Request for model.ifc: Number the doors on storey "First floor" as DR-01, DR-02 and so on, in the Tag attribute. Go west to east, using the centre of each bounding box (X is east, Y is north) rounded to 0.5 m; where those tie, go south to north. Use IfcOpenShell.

First a look at what the model holds.

```python
import ifcopenshell
import ifcopenshell.util.element
import ifcopenshell.util.placement

model = ifcopenshell.open("model.ifc")
print(model.schema)
storey = next(s for s in model.by_type("IfcBuildingStorey") if s.Name == "First floor")
doors = [e for e in ifcopenshell.util.element.get_decomposition(storey) if e.is_a("IfcDoor")]
for e in sorted(doors, key=lambda e: e.id()):
    origin = ifcopenshell.util.placement.get_local_placement(e.ObjectPlacement)[:3, 3]
    print(e.id(), e.Tag, e.Name, origin.round(2) + 0.0, sep=" | ")
```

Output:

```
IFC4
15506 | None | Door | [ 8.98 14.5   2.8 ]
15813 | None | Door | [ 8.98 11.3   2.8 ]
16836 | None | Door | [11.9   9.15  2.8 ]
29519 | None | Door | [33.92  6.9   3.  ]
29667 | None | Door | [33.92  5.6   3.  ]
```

```python
import ifcopenshell
import ifcopenshell.geom
import ifcopenshell.util.element
import ifcopenshell.util.shape

model = ifcopenshell.open("model.ifc")
settings = ifcopenshell.geom.settings()
settings.set("use-world-coords", True)


def centre(element):
    shape = ifcopenshell.geom.create_shape(settings, element)
    return ifcopenshell.util.shape.get_bbox_centroid(shape.geometry)


storey = next(s for s in model.by_type("IfcBuildingStorey") if s.Name == "First floor")
doors = [e for e in ifcopenshell.util.element.get_decomposition(storey) if e.is_a("IfcDoor")]

# Insertion points can sit at a corner or the storey origin, so sort by the geometry (in metres).
centres = {e: centre(e) for e in doors}
doors.sort(key=lambda e: (round(centres[e][0] / 0.5), centres[e][1]))

for i, e in enumerate(doors, start=1):
    number = f"DR-{i:02d}"
    e.Tag = number
    print(e.id(), number)

model.write("model-out.ifc")
```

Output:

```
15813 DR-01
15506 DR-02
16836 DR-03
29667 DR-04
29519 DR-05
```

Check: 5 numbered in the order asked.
